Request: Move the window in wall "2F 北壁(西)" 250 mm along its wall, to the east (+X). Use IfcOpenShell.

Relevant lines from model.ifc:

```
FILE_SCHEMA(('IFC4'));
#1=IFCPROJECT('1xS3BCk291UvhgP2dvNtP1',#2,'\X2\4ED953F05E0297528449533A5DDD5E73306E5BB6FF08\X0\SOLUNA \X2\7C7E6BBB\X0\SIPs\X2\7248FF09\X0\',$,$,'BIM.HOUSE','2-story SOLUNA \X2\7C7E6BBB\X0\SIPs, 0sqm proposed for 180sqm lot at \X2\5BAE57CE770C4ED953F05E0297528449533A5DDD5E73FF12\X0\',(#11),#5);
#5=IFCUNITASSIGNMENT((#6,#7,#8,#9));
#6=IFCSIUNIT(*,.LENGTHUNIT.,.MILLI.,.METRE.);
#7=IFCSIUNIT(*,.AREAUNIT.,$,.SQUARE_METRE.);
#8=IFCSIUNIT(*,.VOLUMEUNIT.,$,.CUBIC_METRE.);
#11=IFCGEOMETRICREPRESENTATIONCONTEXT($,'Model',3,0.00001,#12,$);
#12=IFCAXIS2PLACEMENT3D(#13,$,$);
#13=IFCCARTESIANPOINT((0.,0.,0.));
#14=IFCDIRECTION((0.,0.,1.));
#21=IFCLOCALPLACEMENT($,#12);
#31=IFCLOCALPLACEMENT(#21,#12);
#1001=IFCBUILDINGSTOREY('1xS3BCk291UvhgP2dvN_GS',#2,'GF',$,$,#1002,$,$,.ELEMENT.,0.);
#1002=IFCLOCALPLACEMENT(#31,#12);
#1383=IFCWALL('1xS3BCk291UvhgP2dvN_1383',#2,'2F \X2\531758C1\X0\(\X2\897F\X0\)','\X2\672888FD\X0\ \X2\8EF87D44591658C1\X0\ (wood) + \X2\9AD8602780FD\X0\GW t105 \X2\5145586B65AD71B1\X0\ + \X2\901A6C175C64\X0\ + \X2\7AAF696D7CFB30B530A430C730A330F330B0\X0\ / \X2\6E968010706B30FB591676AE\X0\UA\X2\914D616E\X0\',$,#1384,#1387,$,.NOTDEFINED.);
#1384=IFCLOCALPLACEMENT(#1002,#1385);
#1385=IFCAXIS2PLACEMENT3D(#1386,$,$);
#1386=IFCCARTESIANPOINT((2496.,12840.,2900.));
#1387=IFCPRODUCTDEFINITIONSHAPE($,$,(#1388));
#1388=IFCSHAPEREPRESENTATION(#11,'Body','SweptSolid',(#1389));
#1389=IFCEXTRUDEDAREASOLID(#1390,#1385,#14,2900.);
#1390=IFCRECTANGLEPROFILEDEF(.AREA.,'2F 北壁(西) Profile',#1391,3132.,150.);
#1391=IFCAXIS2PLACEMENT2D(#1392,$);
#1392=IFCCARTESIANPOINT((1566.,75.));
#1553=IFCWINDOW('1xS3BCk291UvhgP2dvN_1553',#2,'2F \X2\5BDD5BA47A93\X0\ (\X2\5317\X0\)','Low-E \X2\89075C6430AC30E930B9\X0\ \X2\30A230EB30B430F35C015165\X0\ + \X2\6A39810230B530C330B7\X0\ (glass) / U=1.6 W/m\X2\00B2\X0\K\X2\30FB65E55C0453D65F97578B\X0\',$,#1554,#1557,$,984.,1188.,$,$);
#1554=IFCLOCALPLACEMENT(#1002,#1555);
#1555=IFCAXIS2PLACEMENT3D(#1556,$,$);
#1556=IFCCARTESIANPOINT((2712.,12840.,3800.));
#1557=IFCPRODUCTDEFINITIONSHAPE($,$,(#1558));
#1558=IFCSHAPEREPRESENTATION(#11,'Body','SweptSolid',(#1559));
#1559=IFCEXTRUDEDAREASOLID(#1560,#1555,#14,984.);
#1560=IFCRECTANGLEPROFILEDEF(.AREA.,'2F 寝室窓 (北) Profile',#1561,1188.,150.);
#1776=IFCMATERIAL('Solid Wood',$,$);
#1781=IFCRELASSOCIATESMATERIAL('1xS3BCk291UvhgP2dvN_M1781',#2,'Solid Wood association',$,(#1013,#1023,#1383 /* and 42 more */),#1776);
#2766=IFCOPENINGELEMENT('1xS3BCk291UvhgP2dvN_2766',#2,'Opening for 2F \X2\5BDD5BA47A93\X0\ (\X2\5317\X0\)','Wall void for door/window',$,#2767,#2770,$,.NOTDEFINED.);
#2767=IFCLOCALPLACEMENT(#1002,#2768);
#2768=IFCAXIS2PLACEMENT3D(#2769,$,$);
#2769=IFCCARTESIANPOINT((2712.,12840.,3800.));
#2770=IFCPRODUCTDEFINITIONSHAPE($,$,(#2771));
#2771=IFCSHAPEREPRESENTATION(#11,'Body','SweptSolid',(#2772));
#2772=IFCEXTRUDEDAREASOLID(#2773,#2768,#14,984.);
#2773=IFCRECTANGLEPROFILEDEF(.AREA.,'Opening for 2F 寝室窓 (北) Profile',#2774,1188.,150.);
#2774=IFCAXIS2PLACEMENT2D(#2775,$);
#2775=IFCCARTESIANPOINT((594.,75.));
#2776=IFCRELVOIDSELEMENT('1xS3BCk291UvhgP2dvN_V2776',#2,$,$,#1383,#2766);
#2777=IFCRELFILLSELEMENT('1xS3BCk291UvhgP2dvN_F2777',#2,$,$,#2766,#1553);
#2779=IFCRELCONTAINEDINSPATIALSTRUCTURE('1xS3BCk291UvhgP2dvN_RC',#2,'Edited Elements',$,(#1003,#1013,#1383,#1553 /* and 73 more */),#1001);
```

```python
import ifcopenshell
import ifcopenshell.api.geometry
import ifcopenshell.util.placement
import ifcopenshell.util.unit

model = ifcopenshell.open("model.ifc")
unit_scale = ifcopenshell.util.unit.calculate_unit_scale(model)

window = model.by_id(1553)
opening = window.FillsVoids[0].RelatingOpeningElement
wall = opening.VoidsElements[0].RelatingBuildingElement

wall_matrix = ifcopenshell.util.placement.get_local_placement(wall.ObjectPlacement)
shift = wall_matrix[:3, 0] * 0.25 / unit_scale
before = ifcopenshell.util.placement.get_local_placement(window.ObjectPlacement)[:3, 3].copy()

# The window is not placed relative to its opening, so move both.
for product in (opening, window):
    matrix = ifcopenshell.util.placement.get_local_placement(product.ObjectPlacement)
    matrix[:3, 3] += shift
    ifcopenshell.api.geometry.edit_object_placement(model, product=product, matrix=matrix, is_si=False)

after = ifcopenshell.util.placement.get_local_placement(window.ObjectPlacement)[:3, 3]
print("window moved by", (after - before).round(3) + 0.0)

model.write("model_rev.ifc")
```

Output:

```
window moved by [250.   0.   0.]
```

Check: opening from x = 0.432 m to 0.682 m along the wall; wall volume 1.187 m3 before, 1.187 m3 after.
